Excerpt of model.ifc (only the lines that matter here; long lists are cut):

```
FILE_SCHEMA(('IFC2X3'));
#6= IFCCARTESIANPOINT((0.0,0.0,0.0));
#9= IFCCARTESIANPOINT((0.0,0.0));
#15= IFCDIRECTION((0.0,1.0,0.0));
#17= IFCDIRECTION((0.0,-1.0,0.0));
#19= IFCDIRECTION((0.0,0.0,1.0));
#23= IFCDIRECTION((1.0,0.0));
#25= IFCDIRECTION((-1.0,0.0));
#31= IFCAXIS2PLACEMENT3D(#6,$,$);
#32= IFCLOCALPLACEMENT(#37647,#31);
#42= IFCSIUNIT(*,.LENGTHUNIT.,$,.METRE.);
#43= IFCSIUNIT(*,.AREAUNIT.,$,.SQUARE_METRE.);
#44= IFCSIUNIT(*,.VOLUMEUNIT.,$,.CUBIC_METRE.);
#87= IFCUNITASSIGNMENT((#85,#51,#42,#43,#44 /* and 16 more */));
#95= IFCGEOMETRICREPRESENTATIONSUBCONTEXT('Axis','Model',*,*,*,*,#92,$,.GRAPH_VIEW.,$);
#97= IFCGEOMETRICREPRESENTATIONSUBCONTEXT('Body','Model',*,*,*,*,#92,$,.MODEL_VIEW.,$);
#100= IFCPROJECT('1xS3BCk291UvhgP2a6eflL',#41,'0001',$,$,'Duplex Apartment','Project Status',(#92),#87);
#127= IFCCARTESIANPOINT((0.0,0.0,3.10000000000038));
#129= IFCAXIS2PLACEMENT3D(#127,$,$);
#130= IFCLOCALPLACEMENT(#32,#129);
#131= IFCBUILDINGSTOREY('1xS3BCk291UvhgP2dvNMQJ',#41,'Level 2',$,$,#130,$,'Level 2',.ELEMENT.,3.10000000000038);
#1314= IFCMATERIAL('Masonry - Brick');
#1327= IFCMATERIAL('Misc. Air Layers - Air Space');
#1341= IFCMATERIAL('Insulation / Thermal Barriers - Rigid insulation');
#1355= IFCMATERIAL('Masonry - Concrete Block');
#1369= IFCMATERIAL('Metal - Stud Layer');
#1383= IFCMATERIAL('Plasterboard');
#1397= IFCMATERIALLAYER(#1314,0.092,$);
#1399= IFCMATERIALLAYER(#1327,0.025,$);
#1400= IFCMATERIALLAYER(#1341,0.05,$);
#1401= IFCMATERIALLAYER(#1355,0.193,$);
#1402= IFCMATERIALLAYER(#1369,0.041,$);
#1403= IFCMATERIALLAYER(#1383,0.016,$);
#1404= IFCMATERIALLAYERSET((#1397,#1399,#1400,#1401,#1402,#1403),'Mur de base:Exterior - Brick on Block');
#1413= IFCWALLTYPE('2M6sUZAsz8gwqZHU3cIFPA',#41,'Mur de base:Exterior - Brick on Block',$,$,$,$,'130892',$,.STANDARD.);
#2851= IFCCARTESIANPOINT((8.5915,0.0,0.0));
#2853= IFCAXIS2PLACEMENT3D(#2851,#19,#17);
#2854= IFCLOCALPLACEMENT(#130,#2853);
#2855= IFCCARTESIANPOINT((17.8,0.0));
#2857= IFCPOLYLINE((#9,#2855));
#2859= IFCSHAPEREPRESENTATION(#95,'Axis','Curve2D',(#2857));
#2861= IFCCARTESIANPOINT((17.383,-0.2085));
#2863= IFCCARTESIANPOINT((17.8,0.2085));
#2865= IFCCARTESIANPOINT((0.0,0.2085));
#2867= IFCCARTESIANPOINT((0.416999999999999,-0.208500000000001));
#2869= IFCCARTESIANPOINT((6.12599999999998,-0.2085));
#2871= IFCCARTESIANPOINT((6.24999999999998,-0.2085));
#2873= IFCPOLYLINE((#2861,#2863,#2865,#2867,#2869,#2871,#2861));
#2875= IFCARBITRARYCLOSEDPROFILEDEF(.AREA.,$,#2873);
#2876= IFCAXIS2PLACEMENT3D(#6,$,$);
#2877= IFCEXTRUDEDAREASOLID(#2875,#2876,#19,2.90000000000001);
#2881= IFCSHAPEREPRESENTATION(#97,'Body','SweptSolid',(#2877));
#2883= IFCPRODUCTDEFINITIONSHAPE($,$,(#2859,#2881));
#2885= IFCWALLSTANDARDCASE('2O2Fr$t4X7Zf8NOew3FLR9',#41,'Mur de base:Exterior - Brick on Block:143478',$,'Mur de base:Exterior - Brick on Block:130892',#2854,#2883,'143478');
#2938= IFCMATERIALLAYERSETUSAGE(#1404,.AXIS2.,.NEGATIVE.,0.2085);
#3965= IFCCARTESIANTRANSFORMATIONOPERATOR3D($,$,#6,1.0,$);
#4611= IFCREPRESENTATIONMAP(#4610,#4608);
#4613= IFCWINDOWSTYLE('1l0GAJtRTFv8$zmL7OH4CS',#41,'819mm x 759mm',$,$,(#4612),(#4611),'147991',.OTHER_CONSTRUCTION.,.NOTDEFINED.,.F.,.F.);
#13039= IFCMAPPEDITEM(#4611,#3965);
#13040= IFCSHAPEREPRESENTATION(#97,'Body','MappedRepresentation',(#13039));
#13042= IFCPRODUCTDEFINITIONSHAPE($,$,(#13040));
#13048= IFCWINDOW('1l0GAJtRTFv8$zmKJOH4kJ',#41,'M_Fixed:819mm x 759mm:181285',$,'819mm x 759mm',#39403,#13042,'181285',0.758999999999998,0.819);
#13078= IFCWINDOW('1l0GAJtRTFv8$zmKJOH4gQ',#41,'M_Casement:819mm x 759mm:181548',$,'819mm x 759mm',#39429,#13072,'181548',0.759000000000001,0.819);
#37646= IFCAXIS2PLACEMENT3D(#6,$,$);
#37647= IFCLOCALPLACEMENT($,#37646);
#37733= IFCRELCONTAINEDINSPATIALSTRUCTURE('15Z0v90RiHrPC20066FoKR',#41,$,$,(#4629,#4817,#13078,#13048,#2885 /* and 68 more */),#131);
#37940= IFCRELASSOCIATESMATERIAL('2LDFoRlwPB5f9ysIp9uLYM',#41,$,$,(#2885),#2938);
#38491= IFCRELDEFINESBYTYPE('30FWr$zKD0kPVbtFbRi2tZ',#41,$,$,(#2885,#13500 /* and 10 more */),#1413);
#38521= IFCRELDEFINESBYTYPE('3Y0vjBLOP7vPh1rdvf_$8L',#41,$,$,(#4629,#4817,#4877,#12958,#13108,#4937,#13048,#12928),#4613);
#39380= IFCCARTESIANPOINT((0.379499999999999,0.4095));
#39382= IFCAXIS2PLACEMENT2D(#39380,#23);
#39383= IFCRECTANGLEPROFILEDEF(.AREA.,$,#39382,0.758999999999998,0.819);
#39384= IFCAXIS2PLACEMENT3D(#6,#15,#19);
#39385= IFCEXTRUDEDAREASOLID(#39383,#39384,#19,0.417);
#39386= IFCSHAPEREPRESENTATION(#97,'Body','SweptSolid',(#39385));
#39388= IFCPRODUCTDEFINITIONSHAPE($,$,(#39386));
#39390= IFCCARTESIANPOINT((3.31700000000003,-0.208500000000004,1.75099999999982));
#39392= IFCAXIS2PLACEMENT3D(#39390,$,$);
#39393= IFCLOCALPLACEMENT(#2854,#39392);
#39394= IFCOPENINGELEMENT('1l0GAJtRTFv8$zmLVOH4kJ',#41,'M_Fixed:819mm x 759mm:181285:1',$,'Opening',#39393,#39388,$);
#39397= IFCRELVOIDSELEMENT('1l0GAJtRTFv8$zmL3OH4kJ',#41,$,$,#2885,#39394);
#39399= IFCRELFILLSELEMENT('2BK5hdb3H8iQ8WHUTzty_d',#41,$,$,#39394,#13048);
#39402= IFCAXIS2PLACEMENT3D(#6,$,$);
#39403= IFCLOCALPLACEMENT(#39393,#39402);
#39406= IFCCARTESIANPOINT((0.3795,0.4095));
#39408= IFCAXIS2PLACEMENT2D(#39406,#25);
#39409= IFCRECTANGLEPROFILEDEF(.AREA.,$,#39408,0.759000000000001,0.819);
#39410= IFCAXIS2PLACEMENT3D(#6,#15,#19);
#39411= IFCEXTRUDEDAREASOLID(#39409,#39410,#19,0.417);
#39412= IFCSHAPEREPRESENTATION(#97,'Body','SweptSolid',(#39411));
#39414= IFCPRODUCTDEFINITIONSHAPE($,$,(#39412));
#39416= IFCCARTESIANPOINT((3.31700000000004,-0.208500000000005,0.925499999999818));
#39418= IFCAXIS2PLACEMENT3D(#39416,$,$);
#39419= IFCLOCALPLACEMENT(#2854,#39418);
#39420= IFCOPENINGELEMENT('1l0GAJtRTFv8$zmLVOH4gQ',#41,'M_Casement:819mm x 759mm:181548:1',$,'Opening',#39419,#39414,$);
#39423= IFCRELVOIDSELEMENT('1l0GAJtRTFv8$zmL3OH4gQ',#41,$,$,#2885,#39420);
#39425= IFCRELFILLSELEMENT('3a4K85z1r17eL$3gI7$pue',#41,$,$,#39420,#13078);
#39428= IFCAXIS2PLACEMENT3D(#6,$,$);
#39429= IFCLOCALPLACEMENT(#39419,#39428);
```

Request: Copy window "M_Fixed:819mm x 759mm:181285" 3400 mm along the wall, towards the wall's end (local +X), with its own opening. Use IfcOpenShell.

```python
import ifcopenshell
import ifcopenshell.api.feature
import ifcopenshell.api.geometry
import ifcopenshell.api.root
import ifcopenshell.geom
import ifcopenshell.util.element
import ifcopenshell.util.placement
import ifcopenshell.util.shape
import ifcopenshell.util.unit

model = ifcopenshell.open("model.ifc")
unit_scale = ifcopenshell.util.unit.calculate_unit_scale(model)
settings = ifcopenshell.geom.settings()


def volume(element):
    """Net volume in cubic metres, openings subtracted."""
    shape = ifcopenshell.geom.create_shape(settings, element)
    return ifcopenshell.util.shape.get_volume(shape.geometry)


def reuse_history(source, copy):
    """copy_class also copies each property set's owner history, people and application; keep the originals."""
    for rel in copy.IsDefinedBy:
        if rel.is_a("IfcRelDefinesByProperties") and (history := rel.RelatingPropertyDefinition.OwnerHistory):
            rel.RelatingPropertyDefinition.OwnerHistory = source.OwnerHistory
            ifcopenshell.util.element.remove_deep2(model, history)


window = model.by_guid("1l0GAJtRTFv8$zmKJOH4kJ")
opening = window.FillsVoids[0].RelatingOpeningElement
wall = opening.VoidsElements[0].RelatingBuildingElement
before = volume(wall)
shift = ifcopenshell.util.placement.get_local_placement(wall.ObjectPlacement)[:3, 0] * 3.4 / unit_scale

# copy_class copies the void relationship, type, container and properties, but no geometry.
new_opening = ifcopenshell.api.root.copy_class(model, product=opening)
new_opening.Representation = ifcopenshell.util.element.copy_deep(
    model, opening.Representation, exclude=["IfcGeometricRepresentationContext", "IfcRepresentationMap"]
)
new_opening.Name = "M_Fixed:819mm x 759mm"
new_window = ifcopenshell.api.root.copy_class(model, product=window)
new_window.Representation = ifcopenshell.util.element.copy_deep(
    model, window.Representation, exclude=["IfcGeometricRepresentationContext", "IfcRepresentationMap"]
)
new_window.Name = "M_Fixed:819mm x 759mm"
new_window.Tag = None
reuse_history(window, new_window)
fills = ifcopenshell.api.feature.add_filling(model, opening=new_opening, element=new_window)
fills.OwnerHistory = new_window.OwnerHistory  # required in IFC2X3

for old, new in ((opening, new_opening), (window, new_window)):
    matrix = ifcopenshell.util.placement.get_local_placement(old.ObjectPlacement)
    matrix[:3, 3] += shift
    ifcopenshell.api.geometry.edit_object_placement(model, product=new, matrix=matrix, is_si=False)

after = volume(wall)

print(f"wall volume {before:.3f} -> {after:.3f} m3")

model.write("model_v2.ifc")
```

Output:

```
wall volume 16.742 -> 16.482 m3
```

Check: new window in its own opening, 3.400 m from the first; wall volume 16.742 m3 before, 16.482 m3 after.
